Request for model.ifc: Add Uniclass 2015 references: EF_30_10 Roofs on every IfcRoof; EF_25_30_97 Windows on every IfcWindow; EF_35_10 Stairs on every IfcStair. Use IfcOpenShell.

First a look at what the model holds.

```python
import ifcopenshell

model = ifcopenshell.open("model.ifc")
print(model.schema)
print("classifications:", [c.Name for c in model.by_type("IfcClassification")])
for ifc_class in ("IfcDoor", "IfcRoof", "IfcStair", "IfcWall", "IfcWindow"):
    print(ifc_class, len(model.by_type(ifc_class)))
```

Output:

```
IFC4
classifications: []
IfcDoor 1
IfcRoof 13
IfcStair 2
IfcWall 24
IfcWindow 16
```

```python
import ifcopenshell
import ifcopenshell.api.classification

model = ifcopenshell.open("model.ifc")

system = ifcopenshell.api.classification.add_classification(model, classification="Uniclass 2015")

codes = {
    "IfcRoof": ("EF_30_10", "Roofs"),
    "IfcWindow": ("EF_25_30_97", "Windows"),
    "IfcStair": ("EF_35_10", "Stairs"),
}
for ifc_class, (code, name) in codes.items():
    products = model.by_type(ifc_class)
    ifcopenshell.api.classification.add_reference(
        model, products=products, classification=system, identification=code, name=name
    )
    print(code, len(products))

model.write("model-out.ifc")
```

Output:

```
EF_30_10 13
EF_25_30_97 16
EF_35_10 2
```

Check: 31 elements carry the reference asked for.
